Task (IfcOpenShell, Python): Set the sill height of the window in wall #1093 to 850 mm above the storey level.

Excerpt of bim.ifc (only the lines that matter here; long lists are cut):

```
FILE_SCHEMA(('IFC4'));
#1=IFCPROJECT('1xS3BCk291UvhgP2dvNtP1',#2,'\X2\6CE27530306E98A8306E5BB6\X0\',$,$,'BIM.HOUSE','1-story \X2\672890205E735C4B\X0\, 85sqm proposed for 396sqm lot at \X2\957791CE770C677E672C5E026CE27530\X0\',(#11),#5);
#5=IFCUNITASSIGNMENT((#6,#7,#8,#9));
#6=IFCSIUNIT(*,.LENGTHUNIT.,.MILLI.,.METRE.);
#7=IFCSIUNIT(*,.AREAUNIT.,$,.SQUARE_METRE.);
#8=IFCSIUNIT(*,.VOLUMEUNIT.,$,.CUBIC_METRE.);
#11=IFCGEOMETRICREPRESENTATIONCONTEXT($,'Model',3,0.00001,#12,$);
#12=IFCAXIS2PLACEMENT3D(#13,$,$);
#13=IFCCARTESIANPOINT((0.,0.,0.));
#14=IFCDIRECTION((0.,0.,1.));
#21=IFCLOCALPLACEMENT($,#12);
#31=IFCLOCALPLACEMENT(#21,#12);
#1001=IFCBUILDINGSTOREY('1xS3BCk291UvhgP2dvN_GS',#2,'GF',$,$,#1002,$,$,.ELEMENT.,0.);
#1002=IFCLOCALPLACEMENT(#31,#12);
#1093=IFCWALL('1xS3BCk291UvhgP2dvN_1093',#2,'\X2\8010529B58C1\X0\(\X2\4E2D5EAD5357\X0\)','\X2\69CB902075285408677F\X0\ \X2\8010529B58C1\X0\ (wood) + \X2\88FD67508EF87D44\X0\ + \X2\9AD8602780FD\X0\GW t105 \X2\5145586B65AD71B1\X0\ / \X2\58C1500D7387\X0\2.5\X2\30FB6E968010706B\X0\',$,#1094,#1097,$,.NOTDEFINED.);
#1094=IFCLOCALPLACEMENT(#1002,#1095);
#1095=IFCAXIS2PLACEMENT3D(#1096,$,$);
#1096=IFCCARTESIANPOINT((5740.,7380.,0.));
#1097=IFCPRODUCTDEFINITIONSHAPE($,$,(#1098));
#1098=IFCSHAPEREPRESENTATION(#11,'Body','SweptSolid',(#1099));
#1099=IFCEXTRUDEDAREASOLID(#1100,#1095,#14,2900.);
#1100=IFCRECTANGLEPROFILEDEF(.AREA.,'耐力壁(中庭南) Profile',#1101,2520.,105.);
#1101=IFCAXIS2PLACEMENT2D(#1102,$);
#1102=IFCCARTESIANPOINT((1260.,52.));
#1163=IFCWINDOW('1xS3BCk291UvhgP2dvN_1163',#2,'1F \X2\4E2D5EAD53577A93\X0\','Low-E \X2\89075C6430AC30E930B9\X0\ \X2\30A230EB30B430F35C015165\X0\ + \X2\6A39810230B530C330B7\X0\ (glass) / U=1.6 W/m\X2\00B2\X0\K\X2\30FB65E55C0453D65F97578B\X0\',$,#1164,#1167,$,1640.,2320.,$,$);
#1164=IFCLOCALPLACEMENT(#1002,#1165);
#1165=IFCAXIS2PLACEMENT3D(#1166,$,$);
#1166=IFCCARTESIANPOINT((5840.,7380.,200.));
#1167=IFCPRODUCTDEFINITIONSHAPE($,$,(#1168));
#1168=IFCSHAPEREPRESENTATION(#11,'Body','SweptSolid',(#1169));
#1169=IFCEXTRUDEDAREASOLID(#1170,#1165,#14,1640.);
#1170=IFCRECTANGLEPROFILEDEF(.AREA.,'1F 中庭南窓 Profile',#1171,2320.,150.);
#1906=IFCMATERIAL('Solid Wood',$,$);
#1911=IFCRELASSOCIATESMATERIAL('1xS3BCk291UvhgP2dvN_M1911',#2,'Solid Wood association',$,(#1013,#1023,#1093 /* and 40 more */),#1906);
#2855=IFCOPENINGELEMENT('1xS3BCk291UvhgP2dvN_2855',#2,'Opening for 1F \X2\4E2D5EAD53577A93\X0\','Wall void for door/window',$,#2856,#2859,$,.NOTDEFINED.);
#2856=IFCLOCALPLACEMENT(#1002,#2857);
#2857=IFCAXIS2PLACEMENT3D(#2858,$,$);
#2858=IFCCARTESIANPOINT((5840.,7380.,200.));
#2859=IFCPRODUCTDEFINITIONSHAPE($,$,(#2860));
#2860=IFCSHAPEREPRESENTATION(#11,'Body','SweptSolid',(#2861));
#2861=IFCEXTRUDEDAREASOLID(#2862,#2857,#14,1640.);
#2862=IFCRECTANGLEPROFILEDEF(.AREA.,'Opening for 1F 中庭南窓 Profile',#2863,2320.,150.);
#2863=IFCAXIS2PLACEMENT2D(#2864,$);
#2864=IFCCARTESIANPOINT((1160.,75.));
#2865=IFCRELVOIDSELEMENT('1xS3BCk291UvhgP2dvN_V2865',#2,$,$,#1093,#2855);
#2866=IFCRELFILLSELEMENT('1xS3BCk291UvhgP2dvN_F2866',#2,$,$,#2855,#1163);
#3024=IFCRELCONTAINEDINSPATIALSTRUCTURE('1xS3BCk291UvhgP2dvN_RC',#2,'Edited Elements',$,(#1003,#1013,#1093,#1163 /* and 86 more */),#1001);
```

```python
import numpy as np
import ifcopenshell
import ifcopenshell.api.geometry
import ifcopenshell.geom
import ifcopenshell.util.element
import ifcopenshell.util.placement
import ifcopenshell.util.shape
import ifcopenshell.util.unit

model = ifcopenshell.open("bim.ifc")
unit_scale = ifcopenshell.util.unit.calculate_unit_scale(model)

window = model.by_guid("1xS3BCk291UvhgP2dvN_1163")
opening = window.FillsVoids[0].RelatingOpeningElement
storey = ifcopenshell.util.element.get_container(window, ifc_class="IfcBuildingStorey")
level = ifcopenshell.util.placement.get_local_placement(storey.ObjectPlacement)[2, 3]

# The opening's origin need not be at the sill, so measure its lowest point.
shape = ifcopenshell.geom.create_shape(ifcopenshell.geom.settings(), opening)
bottom = ifcopenshell.util.shape.get_shape_bottom_elevation(shape, shape.geometry) / unit_scale
dz = level + 850.0 - bottom

shift = np.array([0.0, 0.0, dz])
# The window is not placed relative to its opening, so move both.
for product in (opening, window):
    matrix = ifcopenshell.util.placement.get_local_placement(product.ObjectPlacement)
    matrix[:3, 3] += shift
    ifcopenshell.api.geometry.edit_object_placement(model, product=product, matrix=matrix, is_si=False)

print(f"moved by {dz * unit_scale:+.3f} m")

model.write("bim_rev.ifc")
```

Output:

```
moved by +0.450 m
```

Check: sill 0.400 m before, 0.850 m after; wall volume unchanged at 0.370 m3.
